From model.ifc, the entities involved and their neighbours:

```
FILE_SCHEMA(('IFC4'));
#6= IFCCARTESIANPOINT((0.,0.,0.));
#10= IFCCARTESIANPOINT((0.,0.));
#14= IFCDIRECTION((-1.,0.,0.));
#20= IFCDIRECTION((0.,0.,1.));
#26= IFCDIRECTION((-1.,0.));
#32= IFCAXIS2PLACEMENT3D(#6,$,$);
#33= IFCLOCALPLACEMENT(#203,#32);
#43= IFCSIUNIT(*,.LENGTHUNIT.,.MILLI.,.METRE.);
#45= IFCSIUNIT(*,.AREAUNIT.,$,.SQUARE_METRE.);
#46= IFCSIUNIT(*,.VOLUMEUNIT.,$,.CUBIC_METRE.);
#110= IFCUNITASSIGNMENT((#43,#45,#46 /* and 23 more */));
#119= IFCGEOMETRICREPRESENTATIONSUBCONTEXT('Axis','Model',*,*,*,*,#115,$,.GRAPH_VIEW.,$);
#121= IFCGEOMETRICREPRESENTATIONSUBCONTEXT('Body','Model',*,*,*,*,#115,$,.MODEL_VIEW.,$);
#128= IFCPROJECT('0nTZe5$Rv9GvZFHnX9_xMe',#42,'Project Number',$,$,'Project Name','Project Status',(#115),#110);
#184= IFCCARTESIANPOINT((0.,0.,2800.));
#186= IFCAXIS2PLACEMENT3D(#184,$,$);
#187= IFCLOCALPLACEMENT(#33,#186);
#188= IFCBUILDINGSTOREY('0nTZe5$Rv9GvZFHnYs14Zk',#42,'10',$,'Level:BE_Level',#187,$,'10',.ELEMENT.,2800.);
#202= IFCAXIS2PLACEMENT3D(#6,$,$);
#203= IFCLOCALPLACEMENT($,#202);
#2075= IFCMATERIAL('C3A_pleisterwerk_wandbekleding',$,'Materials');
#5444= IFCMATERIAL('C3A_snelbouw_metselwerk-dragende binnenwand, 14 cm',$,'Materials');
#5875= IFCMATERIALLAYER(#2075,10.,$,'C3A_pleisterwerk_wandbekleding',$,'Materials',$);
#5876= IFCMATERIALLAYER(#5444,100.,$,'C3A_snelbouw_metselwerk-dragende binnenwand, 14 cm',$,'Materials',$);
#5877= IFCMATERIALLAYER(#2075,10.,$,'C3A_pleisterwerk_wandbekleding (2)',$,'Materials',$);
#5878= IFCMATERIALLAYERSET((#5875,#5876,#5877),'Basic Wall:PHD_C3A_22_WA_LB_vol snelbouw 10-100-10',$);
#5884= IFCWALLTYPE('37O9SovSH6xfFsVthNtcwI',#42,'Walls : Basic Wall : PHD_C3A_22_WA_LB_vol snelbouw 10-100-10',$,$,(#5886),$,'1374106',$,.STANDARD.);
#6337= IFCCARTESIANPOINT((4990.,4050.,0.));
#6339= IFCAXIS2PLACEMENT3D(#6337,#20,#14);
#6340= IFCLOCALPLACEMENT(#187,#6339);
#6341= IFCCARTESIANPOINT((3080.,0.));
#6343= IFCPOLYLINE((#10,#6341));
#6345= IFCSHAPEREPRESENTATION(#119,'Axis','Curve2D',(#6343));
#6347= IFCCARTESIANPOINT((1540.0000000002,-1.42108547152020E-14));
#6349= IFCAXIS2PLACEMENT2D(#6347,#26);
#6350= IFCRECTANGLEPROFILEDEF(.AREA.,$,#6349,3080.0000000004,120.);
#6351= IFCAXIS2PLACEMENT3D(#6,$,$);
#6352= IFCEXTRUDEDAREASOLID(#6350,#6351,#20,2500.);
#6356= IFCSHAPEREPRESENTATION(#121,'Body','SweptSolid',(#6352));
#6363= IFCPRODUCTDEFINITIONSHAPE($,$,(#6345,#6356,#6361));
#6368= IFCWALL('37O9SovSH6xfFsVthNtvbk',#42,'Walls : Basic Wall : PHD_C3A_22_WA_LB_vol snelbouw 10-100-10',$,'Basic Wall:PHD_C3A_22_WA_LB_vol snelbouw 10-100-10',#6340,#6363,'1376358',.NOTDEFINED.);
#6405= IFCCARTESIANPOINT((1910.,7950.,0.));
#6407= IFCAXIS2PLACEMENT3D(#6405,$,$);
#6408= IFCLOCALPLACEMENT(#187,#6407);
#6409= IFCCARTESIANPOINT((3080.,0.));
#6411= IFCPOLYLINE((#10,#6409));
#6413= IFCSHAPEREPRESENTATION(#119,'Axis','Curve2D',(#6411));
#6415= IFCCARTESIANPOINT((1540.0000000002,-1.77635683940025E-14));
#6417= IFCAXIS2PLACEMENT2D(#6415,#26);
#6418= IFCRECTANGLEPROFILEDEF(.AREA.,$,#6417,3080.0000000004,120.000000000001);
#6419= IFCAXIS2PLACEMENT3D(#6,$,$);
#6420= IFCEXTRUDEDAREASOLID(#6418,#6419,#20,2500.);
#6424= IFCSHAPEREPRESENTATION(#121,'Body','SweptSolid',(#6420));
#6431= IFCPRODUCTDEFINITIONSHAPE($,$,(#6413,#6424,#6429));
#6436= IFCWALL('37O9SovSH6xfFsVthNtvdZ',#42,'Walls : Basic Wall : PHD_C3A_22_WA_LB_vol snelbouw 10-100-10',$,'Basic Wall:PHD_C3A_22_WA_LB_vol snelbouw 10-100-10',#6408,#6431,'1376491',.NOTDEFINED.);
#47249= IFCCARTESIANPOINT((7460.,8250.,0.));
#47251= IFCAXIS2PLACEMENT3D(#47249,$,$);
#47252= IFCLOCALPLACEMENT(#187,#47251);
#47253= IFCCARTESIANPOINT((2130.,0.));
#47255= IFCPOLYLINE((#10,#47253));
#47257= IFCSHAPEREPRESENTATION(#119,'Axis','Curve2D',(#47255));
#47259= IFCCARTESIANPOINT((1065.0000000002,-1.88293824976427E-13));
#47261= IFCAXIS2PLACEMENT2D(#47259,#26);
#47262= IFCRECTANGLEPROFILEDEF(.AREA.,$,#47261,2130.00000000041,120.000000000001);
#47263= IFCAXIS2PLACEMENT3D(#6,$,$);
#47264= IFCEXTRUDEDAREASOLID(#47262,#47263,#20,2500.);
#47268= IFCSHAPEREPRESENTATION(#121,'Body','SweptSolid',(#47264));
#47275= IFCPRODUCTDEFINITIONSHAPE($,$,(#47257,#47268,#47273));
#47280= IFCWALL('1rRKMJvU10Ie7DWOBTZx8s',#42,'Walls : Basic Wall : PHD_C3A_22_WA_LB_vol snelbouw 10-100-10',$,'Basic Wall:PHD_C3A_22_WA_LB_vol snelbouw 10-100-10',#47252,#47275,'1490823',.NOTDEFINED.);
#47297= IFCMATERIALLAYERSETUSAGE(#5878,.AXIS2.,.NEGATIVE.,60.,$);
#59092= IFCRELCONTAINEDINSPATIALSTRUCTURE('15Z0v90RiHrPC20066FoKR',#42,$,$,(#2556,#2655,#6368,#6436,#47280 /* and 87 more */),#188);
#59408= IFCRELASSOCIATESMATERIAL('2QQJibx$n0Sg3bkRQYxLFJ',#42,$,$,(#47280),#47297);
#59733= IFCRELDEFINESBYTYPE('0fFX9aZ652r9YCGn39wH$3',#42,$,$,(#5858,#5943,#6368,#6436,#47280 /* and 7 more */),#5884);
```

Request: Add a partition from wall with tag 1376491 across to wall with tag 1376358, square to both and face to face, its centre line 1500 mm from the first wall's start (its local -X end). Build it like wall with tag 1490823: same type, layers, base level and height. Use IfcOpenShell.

```python
import numpy as np
import ifcopenshell
import ifcopenshell.api.geometry
import ifcopenshell.api.material
import ifcopenshell.api.pset
import ifcopenshell.api.root
import ifcopenshell.api.spatial
import ifcopenshell.api.type
import ifcopenshell.geom
import ifcopenshell.util.element
import ifcopenshell.util.placement
import ifcopenshell.util.representation
import ifcopenshell.util.shape
import ifcopenshell.util.unit

model = ifcopenshell.open("model.ifc")
unit_scale = ifcopenshell.util.unit.calculate_unit_scale(model)
settings = ifcopenshell.geom.settings()
settings.set("use-world-coords", True)

start_wall = model.by_guid("37O9SovSH6xfFsVthNtvdZ")
end_wall = model.by_guid("37O9SovSH6xfFsVthNtvbk")
like = model.by_id(47280)
matrix = ifcopenshell.util.placement.get_local_placement(start_wall.ObjectPlacement)
matrix[:3, 3] *= unit_scale


def extent(element):
    """Bounding box in the first wall's axes, in metres."""
    shape = ifcopenshell.geom.create_shape(settings, element)
    points = (ifcopenshell.util.shape.get_vertices(shape.geometry) - matrix[:3, 3]) @ matrix[:3, :3]
    return points.min(axis=0), points.max(axis=0)


y_start = extent(start_wall)[0][1]
y_end = extent(end_wall)[1][1]
like_min, like_max = extent(like)
length, height = float(abs(y_end - y_start)), float(like_max[2] - like_min[2])
layer_set = ifcopenshell.util.element.get_material(like, should_skip_usage=True)
thickness = sum(layer.LayerThickness for layer in layer_set.MaterialLayers) * unit_scale

wall = ifcopenshell.api.root.create_entity(model, ifc_class="IfcWall", name="New partition")
storey = ifcopenshell.util.element.get_container(like)
ifcopenshell.api.spatial.assign_container(model, products=[wall], relating_structure=storey)
ifcopenshell.api.type.assign_type(
    model, related_objects=[wall], relating_type=ifcopenshell.util.element.get_type(like), should_map_representations=False
)
rel = ifcopenshell.api.material.assign_material(
    model, products=[wall], type="IfcMaterialLayerSetUsage", material=layer_set
)
rel.RelatingMaterial.OffsetFromReferenceLine = -thickness / 2 / unit_scale
pset = ifcopenshell.api.pset.add_pset(model, product=wall, name="Pset_WallCommon")
ifcopenshell.api.pset.edit_pset(model, pset=pset, properties={"IsExternal": False, "LoadBearing": False})

# The axis runs down the middle of the wall.
axis = ifcopenshell.api.geometry.add_axis_representation(
    model, context=ifcopenshell.util.representation.get_context(model, "Model", "Axis"), axis=[(0.0, 0.0), (length, 0.0)]
)
body = ifcopenshell.api.geometry.add_wall_representation(
    model,
    context=ifcopenshell.util.representation.get_context(model, "Model", "Body", "MODEL_VIEW"),
    length=length,
    height=height,
    thickness=thickness,
    offset=-thickness / 2,
)
for representation in (axis, body):
    ifcopenshell.api.geometry.assign_representation(model, product=wall, representation=representation)

placement = matrix @ ifcopenshell.util.placement.rotation(-90, "Z")
placement[:, 3] = matrix @ np.array([extent(start_wall)[0][0] + 1.5, y_start, like_min[2], 1.0])
ifcopenshell.api.geometry.edit_object_placement(model, product=wall, matrix=placement)

print(f"partition {length:.3f} m long, {height:.3f} m high, {thickness:.3f} m thick")

model.write("model_rev.ifc")
```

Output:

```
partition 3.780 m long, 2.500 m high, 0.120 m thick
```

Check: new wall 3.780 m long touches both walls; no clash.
